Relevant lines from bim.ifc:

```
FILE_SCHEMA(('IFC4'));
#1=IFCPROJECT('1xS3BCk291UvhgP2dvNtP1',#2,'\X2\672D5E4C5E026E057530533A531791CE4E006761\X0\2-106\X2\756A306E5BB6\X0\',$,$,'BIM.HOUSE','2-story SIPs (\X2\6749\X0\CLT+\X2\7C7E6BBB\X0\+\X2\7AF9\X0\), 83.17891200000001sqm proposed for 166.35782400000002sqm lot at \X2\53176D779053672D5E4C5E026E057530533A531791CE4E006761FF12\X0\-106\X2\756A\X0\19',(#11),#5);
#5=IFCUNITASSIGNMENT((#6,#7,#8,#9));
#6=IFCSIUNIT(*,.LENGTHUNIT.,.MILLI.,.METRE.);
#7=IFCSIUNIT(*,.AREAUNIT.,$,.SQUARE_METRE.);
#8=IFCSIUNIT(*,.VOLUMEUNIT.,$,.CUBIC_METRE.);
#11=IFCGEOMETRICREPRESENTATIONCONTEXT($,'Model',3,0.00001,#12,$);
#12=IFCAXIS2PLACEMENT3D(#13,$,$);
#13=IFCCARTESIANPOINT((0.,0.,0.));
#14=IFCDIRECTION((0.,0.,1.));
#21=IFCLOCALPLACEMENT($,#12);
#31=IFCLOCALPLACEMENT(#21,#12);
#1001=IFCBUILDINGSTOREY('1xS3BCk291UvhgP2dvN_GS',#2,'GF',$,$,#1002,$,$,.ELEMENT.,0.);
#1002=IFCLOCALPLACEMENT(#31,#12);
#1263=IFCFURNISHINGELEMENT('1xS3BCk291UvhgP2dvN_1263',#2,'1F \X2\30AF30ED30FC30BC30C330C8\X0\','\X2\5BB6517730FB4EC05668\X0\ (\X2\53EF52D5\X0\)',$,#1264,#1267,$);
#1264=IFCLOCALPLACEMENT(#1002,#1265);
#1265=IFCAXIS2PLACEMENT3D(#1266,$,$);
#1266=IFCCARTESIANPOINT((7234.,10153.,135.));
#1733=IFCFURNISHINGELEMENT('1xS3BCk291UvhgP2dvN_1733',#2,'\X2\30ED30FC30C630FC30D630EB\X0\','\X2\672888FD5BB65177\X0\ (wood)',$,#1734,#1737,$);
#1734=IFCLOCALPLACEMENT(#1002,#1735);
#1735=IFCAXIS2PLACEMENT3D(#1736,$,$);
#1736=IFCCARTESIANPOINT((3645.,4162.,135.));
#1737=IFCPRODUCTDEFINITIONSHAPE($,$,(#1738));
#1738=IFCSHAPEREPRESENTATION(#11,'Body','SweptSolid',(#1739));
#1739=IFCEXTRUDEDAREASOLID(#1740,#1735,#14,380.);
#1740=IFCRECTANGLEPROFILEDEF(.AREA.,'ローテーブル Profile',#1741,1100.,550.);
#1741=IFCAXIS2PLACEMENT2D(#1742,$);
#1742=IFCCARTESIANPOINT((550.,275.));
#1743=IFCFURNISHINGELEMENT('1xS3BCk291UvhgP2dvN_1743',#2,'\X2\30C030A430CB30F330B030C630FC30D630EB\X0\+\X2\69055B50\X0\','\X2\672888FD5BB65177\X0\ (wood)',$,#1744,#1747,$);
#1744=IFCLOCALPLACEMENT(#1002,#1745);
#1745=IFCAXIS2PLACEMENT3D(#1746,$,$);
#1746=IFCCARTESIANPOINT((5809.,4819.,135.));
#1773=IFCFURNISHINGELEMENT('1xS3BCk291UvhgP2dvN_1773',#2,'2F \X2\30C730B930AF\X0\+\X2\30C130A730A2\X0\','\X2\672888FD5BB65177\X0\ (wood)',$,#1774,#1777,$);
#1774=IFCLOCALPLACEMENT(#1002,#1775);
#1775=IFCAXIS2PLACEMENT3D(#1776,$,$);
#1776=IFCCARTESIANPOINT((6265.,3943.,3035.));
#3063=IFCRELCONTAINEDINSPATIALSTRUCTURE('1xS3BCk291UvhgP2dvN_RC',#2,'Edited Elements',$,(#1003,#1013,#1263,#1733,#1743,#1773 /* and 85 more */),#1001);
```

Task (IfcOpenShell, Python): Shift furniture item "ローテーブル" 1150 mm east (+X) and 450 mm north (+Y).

```python
import ifcopenshell
import ifcopenshell.api.geometry
import ifcopenshell.util.placement

model = ifcopenshell.open("bim.ifc")

item = model.by_guid("1xS3BCk291UvhgP2dvN_1733")
matrix = ifcopenshell.util.placement.get_local_placement(item.ObjectPlacement)
matrix[0, 3] += 1150.0
matrix[1, 3] += 450.0
ifcopenshell.api.geometry.edit_object_placement(model, product=item, matrix=matrix, is_si=False)

print(ifcopenshell.util.placement.get_local_placement(item.ObjectPlacement).round(3) + 0.0)

model.write("bim_edited.ifc")
```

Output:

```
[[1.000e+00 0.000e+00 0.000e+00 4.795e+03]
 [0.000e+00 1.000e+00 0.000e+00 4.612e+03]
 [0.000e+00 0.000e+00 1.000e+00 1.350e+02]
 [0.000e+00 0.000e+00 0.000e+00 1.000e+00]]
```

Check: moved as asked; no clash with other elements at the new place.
